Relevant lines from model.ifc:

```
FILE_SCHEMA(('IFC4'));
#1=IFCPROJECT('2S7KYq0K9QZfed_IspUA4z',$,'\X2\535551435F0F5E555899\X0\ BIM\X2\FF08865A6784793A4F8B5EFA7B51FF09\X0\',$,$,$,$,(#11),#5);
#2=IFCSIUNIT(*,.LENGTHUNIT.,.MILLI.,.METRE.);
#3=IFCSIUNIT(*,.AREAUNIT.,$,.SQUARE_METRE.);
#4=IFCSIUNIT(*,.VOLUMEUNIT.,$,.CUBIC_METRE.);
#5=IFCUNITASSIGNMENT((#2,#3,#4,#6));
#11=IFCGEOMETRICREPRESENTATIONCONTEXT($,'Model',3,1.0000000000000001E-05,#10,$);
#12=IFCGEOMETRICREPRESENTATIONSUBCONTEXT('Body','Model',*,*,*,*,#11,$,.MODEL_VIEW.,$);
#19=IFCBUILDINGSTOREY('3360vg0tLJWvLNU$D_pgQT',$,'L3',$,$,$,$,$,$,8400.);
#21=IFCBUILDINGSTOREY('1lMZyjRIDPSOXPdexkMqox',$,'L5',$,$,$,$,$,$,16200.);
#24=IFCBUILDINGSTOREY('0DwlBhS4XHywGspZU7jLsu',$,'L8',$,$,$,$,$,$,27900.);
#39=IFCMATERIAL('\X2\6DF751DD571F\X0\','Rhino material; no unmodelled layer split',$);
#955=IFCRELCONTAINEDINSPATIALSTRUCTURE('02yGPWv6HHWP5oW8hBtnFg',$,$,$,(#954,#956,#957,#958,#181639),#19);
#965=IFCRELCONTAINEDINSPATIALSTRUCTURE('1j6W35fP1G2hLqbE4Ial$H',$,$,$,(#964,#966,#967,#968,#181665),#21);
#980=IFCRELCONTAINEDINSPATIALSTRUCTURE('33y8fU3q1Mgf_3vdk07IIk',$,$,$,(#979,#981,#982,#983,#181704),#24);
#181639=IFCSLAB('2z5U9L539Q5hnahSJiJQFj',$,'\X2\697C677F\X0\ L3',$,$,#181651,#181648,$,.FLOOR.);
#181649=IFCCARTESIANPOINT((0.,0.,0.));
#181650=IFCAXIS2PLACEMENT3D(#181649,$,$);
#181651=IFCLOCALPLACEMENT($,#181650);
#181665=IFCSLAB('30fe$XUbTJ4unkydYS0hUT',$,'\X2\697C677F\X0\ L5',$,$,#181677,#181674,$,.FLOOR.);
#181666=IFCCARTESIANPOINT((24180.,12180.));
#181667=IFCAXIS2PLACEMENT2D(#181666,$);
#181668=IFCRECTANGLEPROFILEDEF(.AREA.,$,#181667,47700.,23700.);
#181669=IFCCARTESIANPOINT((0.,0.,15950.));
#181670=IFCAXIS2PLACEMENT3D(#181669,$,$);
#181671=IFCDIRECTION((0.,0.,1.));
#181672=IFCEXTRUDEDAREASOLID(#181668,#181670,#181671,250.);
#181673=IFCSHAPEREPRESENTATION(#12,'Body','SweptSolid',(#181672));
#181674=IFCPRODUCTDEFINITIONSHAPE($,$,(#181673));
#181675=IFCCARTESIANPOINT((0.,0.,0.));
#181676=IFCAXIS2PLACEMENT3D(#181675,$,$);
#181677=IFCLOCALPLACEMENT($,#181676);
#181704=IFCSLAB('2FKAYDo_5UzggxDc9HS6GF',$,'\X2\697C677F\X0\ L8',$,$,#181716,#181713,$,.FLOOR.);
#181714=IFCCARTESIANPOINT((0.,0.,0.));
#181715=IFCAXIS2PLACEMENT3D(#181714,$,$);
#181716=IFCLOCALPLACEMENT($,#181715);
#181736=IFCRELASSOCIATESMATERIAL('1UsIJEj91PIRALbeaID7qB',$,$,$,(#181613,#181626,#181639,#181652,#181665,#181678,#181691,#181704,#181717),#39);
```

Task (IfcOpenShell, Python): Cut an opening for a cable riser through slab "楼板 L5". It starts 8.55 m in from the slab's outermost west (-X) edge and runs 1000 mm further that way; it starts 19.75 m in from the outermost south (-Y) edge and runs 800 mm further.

```python
import numpy as np
import ifcopenshell
import ifcopenshell.api.feature
import ifcopenshell.api.geometry
import ifcopenshell.api.root
import ifcopenshell.geom
import ifcopenshell.util.placement
import ifcopenshell.util.representation
import ifcopenshell.util.shape
import ifcopenshell.util.unit

model = ifcopenshell.open("model.ifc")
unit_scale = ifcopenshell.util.unit.calculate_unit_scale(model)
settings = ifcopenshell.geom.settings()


def volume(element):
    """Net volume in cubic metres, openings subtracted."""
    shape = ifcopenshell.geom.create_shape(settings, element)
    return ifcopenshell.util.shape.get_volume(shape.geometry)


slab = model.by_guid("30fe$XUbTJ4unkydYS0hUT")
before = volume(slab)

# Extent in the slab's own axes, in metres. The edges named are its -X and -Y sides.
slab_shape = ifcopenshell.geom.create_shape(settings, slab)
vertices = ifcopenshell.util.shape.get_vertices(slab_shape.geometry)
x_min, y_min, bottom = vertices.min(axis=0)
top = vertices[:, 2].max()

opening = ifcopenshell.api.root.create_entity(model, ifc_class="IfcOpeningElement", name="Cable riser opening", predefined_type="OPENING")
context = ifcopenshell.util.representation.get_context(model, "Model", "Body", "MODEL_VIEW")
width, depth = 1, 0.8
outline = [(0.0, 0.0), (width, 0.0), (width, depth), (0.0, depth), (0.0, 0.0)]
# Overshoot both faces by 50 mm so the cut is clean.
shape = ifcopenshell.api.geometry.add_slab_representation(
    model, context=context, depth=top - bottom + 0.1, polyline=outline
)
ifcopenshell.api.geometry.assign_representation(model, product=opening, representation=shape)

matrix = ifcopenshell.util.placement.get_local_placement(slab.ObjectPlacement)
matrix[:, 3] = matrix @ np.append(np.array([x_min + 8.55, y_min + 19.75, bottom - 0.05]) / unit_scale, 1.0)
ifcopenshell.api.geometry.edit_object_placement(model, product=opening, matrix=matrix, is_si=False)
ifcopenshell.api.feature.add_feature(model, feature=opening, element=slab)

after = volume(slab)

print(f"slab volume {before:.3f} -> {after:.3f} m3")

model.write("model_edited.ifc")
```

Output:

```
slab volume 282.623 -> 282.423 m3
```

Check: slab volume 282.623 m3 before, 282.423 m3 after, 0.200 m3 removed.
